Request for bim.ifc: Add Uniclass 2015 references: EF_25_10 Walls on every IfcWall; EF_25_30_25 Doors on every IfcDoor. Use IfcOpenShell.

First a look at what the model holds.

```python
import ifcopenshell

model = ifcopenshell.open("bim.ifc")
print(model.schema)
print("classifications:", [c.Name for c in model.by_type("IfcClassification")])
for ifc_class in ("IfcDoor", "IfcRoof", "IfcStair", "IfcWall", "IfcWindow"):
    print(ifc_class, len(model.by_type(ifc_class)))
```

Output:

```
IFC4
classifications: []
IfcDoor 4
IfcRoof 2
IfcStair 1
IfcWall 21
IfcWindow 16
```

```python
import ifcopenshell
import ifcopenshell.api.classification

model = ifcopenshell.open("bim.ifc")

system = ifcopenshell.api.classification.add_classification(model, classification="Uniclass 2015")

codes = {
    "IfcWall": ("EF_25_10", "Walls"),
    "IfcDoor": ("EF_25_30_25", "Doors"),
}
for ifc_class, (code, name) in codes.items():
    products = model.by_type(ifc_class)
    ifcopenshell.api.classification.add_reference(
        model, products=products, classification=system, identification=code, name=name
    )
    print(code, len(products))

model.write("bim-out.ifc")
```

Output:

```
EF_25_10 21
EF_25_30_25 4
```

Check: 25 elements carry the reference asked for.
